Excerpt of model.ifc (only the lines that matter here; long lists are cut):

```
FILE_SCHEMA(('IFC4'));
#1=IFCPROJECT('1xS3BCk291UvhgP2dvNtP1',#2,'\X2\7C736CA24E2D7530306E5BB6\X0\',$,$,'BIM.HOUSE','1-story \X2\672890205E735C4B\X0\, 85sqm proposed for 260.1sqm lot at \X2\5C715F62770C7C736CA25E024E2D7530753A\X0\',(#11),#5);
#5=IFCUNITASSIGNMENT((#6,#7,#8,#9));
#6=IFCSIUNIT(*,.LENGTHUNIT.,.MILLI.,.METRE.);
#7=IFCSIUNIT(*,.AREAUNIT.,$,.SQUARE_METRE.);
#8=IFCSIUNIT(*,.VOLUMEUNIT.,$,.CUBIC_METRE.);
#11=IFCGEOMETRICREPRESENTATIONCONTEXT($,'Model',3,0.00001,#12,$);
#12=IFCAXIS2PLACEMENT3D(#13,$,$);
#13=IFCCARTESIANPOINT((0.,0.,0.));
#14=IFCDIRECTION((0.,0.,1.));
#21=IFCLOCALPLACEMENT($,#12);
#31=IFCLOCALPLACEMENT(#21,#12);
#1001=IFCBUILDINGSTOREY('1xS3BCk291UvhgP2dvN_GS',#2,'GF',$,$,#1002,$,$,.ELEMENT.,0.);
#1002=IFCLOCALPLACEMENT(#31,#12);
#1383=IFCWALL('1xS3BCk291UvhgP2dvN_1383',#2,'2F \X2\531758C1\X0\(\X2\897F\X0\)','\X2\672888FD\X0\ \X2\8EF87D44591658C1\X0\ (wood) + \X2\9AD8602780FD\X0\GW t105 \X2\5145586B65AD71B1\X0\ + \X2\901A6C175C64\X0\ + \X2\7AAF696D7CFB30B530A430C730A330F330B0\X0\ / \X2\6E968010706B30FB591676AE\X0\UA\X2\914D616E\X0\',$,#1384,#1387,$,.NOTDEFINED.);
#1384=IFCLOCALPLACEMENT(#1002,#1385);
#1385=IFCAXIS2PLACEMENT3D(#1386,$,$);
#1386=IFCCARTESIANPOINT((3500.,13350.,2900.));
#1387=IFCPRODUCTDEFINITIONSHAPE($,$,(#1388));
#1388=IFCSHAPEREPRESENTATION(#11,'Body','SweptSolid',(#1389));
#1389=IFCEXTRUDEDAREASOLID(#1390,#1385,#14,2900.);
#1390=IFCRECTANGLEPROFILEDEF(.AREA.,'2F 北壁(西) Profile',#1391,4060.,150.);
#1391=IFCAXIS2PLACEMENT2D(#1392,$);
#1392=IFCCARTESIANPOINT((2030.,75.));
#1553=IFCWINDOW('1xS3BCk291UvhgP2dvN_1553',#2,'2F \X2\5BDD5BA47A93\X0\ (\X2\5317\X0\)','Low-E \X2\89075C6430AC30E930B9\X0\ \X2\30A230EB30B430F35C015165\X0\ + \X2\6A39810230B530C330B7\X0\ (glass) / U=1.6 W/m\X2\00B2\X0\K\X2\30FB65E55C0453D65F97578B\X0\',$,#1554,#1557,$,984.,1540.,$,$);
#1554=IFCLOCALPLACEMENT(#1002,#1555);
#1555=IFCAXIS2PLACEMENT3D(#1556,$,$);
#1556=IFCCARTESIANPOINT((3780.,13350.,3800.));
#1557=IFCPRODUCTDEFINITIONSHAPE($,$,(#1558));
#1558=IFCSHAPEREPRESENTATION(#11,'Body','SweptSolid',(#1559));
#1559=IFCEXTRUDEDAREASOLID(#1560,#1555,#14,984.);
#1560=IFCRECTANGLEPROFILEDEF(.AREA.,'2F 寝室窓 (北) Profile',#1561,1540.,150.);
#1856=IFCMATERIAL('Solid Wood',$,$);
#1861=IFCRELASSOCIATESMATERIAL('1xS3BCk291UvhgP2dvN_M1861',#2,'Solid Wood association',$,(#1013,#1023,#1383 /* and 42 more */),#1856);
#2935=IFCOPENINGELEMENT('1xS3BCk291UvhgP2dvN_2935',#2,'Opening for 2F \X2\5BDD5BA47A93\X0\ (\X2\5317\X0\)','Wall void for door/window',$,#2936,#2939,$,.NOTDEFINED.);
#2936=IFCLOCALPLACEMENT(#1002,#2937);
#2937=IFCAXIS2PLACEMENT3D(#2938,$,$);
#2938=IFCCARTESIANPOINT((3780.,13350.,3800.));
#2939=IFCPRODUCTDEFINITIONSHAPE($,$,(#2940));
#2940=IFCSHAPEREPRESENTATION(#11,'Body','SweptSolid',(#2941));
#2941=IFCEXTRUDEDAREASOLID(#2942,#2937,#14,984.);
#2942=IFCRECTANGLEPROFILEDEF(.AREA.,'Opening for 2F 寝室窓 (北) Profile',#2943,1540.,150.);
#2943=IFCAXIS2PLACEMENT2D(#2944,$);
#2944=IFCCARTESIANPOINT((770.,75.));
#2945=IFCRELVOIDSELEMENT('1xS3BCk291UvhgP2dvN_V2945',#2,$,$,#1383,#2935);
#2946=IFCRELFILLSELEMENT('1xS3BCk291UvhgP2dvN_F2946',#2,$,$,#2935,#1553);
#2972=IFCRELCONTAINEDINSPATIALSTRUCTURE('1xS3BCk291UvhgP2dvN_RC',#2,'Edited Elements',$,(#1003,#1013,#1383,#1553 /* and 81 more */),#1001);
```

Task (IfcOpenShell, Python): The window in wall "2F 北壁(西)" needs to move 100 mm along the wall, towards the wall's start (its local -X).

```python
import ifcopenshell
import ifcopenshell.api.geometry
import ifcopenshell.util.placement

model = ifcopenshell.open("model.ifc")

window = model.by_id(1553)
opening = window.FillsVoids[0].RelatingOpeningElement
wall = opening.VoidsElements[0].RelatingBuildingElement

wall_matrix = ifcopenshell.util.placement.get_local_placement(wall.ObjectPlacement)
shift = wall_matrix[:3, 0] * -100.0
before = ifcopenshell.util.placement.get_local_placement(window.ObjectPlacement)[:3, 3].copy()

# The window is not placed relative to its opening, so move both.
for product in (opening, window):
    matrix = ifcopenshell.util.placement.get_local_placement(product.ObjectPlacement)
    matrix[:3, 3] += shift
    ifcopenshell.api.geometry.edit_object_placement(model, product=product, matrix=matrix, is_si=False)

after = ifcopenshell.util.placement.get_local_placement(window.ObjectPlacement)[:3, 3]
print("window moved by", (after - before).round(3) + 0.0)

model.write("model_updated.ifc")
```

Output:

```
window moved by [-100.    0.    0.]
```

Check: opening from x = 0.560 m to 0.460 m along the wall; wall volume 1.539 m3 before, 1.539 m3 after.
